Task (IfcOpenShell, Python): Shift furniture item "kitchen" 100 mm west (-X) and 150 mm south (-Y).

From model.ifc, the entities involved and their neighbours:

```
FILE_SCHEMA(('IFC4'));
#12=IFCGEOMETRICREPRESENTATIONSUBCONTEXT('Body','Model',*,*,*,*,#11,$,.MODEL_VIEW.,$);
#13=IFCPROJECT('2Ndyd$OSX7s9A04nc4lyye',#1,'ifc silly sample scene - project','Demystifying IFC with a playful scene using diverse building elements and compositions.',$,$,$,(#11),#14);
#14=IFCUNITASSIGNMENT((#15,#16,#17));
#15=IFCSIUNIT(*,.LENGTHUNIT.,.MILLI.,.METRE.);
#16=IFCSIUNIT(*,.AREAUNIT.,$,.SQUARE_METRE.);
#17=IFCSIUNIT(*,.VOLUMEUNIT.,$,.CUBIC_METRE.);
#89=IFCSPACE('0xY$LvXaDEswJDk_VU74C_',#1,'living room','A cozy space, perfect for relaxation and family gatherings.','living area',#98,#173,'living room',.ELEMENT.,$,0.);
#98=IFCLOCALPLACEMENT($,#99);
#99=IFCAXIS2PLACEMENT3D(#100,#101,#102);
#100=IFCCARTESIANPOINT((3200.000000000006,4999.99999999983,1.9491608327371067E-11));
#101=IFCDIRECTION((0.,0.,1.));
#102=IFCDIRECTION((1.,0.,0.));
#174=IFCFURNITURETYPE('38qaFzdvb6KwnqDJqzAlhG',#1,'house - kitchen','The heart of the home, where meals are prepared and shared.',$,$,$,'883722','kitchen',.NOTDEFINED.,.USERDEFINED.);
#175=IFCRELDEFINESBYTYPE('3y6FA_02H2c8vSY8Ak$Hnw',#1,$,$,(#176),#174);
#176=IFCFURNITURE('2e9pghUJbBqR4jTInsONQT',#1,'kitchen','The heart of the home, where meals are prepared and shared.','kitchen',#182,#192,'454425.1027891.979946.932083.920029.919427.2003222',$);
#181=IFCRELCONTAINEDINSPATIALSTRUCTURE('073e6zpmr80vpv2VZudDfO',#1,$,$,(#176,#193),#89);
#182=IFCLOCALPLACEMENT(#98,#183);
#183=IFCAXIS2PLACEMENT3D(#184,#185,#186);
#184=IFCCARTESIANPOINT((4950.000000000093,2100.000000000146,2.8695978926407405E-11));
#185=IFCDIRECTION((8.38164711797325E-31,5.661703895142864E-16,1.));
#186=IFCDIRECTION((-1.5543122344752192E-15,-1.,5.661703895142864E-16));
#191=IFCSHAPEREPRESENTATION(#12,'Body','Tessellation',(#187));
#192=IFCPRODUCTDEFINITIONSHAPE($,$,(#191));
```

```python
import ifcopenshell
import ifcopenshell.api.geometry
import ifcopenshell.util.placement

model = ifcopenshell.open("model.ifc")

item = model.by_id(176)
matrix = ifcopenshell.util.placement.get_local_placement(item.ObjectPlacement)
matrix[0, 3] -= 100.0
matrix[1, 3] -= 150.0
ifcopenshell.api.geometry.edit_object_placement(model, product=item, matrix=matrix, is_si=False)

print(ifcopenshell.util.placement.get_local_placement(item.ObjectPlacement).round(3) + 0.0)

model.write("model_rev.ifc")
```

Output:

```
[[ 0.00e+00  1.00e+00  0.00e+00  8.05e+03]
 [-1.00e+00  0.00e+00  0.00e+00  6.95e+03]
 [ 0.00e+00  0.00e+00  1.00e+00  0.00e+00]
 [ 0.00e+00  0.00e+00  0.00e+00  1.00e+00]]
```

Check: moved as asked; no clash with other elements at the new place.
